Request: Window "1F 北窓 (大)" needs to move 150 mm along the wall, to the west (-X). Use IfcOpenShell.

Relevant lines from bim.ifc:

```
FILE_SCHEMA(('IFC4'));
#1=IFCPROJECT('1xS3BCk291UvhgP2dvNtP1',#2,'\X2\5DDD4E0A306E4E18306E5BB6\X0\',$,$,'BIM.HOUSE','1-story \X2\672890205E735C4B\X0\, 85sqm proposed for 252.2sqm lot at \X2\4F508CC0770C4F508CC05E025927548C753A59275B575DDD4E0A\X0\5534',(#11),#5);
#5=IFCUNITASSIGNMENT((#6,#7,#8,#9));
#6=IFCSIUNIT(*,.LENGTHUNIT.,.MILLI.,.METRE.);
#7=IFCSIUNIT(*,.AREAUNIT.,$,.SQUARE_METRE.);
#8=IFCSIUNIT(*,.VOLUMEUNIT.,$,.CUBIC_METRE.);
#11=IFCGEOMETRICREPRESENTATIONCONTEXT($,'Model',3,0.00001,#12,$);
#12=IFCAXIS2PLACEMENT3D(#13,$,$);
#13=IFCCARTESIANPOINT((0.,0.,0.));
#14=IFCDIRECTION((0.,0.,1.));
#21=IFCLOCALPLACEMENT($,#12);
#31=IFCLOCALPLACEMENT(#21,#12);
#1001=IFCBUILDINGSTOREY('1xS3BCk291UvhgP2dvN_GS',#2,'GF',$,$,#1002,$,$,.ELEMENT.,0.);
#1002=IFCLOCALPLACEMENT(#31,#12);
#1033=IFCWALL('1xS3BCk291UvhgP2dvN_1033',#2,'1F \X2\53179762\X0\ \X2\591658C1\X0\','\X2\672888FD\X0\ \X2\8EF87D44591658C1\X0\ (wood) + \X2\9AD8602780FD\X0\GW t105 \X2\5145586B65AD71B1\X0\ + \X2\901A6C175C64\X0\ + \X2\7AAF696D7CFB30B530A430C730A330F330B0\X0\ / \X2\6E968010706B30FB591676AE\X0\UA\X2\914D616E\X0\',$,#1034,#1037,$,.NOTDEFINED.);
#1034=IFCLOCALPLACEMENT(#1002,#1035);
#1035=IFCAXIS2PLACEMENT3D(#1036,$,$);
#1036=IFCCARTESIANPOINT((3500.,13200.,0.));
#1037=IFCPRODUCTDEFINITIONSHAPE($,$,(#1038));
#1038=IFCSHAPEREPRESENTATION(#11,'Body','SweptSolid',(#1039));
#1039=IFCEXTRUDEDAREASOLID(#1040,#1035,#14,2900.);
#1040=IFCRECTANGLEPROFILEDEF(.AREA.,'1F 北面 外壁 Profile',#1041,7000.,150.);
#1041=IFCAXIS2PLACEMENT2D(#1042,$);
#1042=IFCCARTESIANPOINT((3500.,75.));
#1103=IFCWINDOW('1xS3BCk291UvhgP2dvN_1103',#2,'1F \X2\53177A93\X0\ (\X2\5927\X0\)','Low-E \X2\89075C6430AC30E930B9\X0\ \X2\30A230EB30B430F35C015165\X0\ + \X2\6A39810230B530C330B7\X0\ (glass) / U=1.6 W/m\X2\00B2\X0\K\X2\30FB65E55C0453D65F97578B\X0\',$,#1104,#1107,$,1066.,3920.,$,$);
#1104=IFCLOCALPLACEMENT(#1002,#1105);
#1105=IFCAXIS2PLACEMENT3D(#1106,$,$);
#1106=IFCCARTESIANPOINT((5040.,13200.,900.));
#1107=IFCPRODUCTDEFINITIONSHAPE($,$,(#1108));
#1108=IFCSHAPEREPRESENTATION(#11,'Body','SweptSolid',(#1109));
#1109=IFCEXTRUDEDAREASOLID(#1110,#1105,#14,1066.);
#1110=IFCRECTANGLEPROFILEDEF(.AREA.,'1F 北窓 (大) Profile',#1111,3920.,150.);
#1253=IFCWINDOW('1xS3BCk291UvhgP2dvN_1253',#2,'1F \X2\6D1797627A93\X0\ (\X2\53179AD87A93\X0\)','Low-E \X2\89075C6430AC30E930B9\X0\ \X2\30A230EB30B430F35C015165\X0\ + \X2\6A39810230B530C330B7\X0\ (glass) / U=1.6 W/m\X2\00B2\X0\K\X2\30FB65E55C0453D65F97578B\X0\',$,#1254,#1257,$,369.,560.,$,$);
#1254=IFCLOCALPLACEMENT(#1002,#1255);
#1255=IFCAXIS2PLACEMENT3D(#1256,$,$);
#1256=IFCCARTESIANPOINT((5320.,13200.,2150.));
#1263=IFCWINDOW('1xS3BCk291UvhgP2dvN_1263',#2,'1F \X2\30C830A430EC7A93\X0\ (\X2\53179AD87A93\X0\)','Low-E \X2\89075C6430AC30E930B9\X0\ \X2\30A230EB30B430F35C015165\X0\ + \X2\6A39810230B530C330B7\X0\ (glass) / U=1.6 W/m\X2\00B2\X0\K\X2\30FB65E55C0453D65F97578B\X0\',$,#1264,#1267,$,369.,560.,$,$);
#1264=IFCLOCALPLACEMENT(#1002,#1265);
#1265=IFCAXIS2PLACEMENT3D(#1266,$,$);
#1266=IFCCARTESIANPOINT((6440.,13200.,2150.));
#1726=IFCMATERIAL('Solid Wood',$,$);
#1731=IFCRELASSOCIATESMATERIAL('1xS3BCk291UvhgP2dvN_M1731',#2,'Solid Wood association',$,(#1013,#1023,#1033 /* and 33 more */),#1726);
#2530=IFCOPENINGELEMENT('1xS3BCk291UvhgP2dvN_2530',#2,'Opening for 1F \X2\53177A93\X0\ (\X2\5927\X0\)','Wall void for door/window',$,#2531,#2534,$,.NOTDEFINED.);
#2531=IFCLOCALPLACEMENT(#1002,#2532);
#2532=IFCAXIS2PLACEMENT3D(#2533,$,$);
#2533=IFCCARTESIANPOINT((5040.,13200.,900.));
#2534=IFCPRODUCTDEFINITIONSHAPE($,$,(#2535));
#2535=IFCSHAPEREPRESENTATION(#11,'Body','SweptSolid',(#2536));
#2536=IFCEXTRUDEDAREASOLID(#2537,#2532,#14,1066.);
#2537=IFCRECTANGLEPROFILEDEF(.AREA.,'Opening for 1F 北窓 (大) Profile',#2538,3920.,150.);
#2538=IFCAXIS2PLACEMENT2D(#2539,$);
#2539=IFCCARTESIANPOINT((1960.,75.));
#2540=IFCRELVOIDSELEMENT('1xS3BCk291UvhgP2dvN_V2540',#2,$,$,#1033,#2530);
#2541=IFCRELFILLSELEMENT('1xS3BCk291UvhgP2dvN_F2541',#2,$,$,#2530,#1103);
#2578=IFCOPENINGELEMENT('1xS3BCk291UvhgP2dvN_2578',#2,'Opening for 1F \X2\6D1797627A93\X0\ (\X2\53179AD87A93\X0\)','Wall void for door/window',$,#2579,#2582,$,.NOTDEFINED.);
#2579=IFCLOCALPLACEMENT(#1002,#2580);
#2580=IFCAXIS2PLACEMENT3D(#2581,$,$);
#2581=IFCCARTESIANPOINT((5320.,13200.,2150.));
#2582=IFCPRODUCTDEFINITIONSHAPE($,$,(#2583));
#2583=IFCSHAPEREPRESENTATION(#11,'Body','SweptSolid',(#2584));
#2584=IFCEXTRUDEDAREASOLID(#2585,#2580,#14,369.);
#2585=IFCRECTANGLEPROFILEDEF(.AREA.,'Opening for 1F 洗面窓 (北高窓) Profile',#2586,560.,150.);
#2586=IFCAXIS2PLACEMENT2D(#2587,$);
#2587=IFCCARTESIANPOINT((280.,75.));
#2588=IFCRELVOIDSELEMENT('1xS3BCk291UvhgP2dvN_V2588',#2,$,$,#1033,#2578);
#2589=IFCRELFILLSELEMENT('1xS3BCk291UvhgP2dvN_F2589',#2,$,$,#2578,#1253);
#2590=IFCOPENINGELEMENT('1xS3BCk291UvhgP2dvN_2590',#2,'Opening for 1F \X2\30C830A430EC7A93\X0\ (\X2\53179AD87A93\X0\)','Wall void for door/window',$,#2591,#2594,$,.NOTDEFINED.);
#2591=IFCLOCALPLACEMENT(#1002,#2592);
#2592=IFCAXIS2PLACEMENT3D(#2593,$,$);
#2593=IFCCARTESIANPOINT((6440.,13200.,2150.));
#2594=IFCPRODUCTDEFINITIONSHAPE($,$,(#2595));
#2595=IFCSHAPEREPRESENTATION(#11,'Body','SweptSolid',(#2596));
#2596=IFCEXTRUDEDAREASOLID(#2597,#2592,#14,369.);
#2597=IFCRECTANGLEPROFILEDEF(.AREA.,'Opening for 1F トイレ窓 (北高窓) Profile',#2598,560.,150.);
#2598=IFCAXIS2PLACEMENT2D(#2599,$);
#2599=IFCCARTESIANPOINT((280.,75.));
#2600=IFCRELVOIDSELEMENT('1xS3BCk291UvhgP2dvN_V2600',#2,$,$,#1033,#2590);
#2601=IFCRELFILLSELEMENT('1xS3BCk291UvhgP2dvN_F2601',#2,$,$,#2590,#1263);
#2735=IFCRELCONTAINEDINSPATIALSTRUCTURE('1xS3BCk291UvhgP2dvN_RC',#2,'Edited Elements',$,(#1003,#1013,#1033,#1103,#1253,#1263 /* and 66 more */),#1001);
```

```python
import ifcopenshell
import ifcopenshell.api.geometry
import ifcopenshell.util.placement

model = ifcopenshell.open("bim.ifc")

window = model.by_guid("1xS3BCk291UvhgP2dvN_1103")
opening = window.FillsVoids[0].RelatingOpeningElement
wall = opening.VoidsElements[0].RelatingBuildingElement

wall_matrix = ifcopenshell.util.placement.get_local_placement(wall.ObjectPlacement)
shift = wall_matrix[:3, 0] * -150.0
before = ifcopenshell.util.placement.get_local_placement(window.ObjectPlacement)[:3, 3].copy()

# The window is not placed relative to its opening, so move both.
for product in (opening, window):
    matrix = ifcopenshell.util.placement.get_local_placement(product.ObjectPlacement)
    matrix[:3, 3] += shift
    ifcopenshell.api.geometry.edit_object_placement(model, product=product, matrix=matrix, is_si=False)

after = ifcopenshell.util.placement.get_local_placement(window.ObjectPlacement)[:3, 3]
print("window moved by", (after - before).round(3) + 0.0)

model.write("bim-out.ifc")
```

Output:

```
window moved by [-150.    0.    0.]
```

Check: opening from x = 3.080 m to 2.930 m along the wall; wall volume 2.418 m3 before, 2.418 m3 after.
